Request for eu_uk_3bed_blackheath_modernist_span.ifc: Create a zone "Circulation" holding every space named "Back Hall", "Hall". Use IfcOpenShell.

First a look at what the model holds.

```python
import ifcopenshell

model = ifcopenshell.open("eu_uk_3bed_blackheath_modernist_span.ifc")
print(model.schema)
seen = {}
for space in model.by_type("IfcSpace"):
    seen[space.LongName] = seen.get(space.LongName, 0) + 1
for name, count in sorted(seen.items(), key=str):
    print(count, "x", name)
print("zones:", [z.Name for z in model.by_type("IfcZone")][:20])
```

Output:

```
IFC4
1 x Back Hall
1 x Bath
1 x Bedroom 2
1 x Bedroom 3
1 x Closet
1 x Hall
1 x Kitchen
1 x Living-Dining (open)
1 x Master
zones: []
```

```python
import ifcopenshell
import ifcopenshell.api.group
import ifcopenshell.api.root

model = ifcopenshell.open("eu_uk_3bed_blackheath_modernist_span.ifc")

names = {"Back Hall", "Hall"}
spaces = [s for s in model.by_type("IfcSpace") if s.LongName in names]

zone = ifcopenshell.api.root.create_entity(model, ifc_class="IfcZone", name="Circulation")
ifcopenshell.api.group.assign_group(model, products=spaces, group=zone)
print(len(spaces), "spaces in", zone.Name)

model.write("eu_uk_3bed_blackheath_modernist_span_updated.ifc")
```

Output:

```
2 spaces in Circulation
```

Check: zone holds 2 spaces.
